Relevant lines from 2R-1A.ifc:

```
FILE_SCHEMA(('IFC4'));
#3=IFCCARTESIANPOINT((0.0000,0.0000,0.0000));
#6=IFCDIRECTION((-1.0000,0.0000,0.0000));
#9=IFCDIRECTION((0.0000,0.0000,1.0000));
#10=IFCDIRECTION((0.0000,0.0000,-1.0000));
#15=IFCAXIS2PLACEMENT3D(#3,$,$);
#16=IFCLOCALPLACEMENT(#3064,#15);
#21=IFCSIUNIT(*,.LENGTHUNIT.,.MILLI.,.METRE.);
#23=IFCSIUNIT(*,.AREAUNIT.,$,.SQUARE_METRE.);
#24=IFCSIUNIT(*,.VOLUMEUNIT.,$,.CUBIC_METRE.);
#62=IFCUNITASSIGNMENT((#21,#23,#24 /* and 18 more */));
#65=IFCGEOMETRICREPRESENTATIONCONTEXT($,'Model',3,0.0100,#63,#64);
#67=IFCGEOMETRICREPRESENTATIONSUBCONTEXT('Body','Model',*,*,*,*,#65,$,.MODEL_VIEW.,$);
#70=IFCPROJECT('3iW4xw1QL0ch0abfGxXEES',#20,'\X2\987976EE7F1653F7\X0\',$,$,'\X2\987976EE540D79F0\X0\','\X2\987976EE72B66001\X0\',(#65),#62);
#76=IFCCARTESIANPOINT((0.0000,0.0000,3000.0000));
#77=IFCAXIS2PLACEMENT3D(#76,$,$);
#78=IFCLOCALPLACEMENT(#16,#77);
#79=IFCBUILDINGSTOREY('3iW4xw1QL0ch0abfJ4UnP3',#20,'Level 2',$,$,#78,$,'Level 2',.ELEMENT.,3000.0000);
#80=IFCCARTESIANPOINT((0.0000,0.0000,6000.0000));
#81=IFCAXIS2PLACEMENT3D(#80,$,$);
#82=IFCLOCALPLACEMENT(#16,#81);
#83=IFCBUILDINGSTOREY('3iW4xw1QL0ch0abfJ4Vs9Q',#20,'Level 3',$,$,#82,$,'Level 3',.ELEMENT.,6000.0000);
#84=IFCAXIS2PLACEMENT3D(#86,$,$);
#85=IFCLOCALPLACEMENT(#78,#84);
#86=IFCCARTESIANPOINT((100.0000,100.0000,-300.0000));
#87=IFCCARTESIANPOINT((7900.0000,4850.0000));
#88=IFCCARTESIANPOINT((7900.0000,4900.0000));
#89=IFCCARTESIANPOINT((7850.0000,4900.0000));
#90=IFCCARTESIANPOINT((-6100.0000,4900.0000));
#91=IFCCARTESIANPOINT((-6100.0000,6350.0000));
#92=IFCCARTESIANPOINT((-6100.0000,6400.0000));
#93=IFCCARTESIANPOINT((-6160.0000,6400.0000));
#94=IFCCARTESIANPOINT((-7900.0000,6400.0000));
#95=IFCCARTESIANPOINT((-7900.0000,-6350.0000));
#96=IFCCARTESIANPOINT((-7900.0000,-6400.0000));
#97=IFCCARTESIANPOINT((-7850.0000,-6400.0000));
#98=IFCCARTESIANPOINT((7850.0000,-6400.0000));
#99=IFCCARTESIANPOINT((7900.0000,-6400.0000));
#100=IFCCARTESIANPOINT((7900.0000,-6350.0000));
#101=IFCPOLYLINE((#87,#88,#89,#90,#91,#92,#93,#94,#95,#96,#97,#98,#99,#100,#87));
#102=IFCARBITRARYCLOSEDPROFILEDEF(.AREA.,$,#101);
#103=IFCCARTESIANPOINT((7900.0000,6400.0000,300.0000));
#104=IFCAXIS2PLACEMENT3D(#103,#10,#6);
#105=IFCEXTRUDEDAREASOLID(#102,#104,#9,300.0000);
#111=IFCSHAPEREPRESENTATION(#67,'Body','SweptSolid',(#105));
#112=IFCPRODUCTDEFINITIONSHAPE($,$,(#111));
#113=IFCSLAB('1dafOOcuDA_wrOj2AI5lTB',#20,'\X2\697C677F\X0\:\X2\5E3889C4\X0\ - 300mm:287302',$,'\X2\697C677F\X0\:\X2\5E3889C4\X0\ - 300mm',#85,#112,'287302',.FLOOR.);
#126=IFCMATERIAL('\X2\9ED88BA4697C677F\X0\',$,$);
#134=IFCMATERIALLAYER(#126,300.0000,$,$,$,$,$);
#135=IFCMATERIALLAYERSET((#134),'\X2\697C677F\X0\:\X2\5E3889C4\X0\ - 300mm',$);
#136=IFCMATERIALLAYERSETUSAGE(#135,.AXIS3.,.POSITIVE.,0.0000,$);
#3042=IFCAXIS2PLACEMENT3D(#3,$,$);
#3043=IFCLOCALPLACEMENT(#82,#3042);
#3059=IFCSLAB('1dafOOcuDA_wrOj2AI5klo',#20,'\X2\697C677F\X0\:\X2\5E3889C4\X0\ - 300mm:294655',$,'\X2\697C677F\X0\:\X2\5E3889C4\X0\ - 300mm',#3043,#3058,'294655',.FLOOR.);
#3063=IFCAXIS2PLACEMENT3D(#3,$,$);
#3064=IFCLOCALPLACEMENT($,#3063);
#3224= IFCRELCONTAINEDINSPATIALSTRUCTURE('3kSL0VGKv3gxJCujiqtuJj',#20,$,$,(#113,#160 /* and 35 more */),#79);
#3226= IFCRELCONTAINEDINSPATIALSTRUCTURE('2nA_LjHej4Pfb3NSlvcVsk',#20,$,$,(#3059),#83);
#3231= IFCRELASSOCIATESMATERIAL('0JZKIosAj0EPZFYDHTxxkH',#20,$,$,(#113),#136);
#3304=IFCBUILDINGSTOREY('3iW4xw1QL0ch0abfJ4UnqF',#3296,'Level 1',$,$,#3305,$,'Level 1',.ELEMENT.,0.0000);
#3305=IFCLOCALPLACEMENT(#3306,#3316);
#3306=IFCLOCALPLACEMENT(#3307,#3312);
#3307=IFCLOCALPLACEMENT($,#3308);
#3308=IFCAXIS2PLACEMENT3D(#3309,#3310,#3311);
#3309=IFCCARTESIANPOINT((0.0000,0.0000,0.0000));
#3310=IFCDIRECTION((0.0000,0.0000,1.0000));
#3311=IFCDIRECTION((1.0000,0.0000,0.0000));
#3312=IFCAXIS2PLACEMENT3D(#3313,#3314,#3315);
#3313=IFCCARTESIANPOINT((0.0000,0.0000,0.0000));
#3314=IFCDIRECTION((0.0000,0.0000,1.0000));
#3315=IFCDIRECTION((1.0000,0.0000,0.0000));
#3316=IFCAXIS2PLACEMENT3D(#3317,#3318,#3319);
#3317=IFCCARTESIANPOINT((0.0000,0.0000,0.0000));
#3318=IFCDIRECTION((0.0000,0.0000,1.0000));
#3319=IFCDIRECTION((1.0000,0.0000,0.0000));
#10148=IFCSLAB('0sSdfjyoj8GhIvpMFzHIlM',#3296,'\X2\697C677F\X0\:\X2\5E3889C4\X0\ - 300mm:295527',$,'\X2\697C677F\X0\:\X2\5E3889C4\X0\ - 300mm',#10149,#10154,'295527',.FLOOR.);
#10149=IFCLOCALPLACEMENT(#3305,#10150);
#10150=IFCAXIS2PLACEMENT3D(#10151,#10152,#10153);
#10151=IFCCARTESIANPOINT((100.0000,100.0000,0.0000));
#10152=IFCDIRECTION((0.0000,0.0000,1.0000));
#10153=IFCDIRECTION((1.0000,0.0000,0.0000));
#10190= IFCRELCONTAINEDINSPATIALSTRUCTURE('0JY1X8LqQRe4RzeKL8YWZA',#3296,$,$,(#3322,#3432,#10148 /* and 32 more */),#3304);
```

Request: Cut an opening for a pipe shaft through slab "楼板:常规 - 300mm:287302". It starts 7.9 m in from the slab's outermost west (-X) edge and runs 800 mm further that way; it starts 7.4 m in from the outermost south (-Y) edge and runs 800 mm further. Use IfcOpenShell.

```python
import numpy as np
import ifcopenshell
import ifcopenshell.api.feature
import ifcopenshell.api.geometry
import ifcopenshell.api.root
import ifcopenshell.geom
import ifcopenshell.util.placement
import ifcopenshell.util.representation
import ifcopenshell.util.shape
import ifcopenshell.util.unit

model = ifcopenshell.open("2R-1A.ifc")
unit_scale = ifcopenshell.util.unit.calculate_unit_scale(model)
settings = ifcopenshell.geom.settings()


def volume(element):
    """Net volume in cubic metres, openings subtracted."""
    shape = ifcopenshell.geom.create_shape(settings, element)
    return ifcopenshell.util.shape.get_volume(shape.geometry)


slab = model.by_guid("1dafOOcuDA_wrOj2AI5lTB")
before = volume(slab)

# Extent in the slab's own axes, in metres. The edges named are its -X and -Y sides.
slab_shape = ifcopenshell.geom.create_shape(settings, slab)
vertices = ifcopenshell.util.shape.get_vertices(slab_shape.geometry)
x_min, y_min, bottom = vertices.min(axis=0)
top = vertices[:, 2].max()

opening = ifcopenshell.api.root.create_entity(model, ifc_class="IfcOpeningElement", name="Pipe shaft opening", predefined_type="OPENING")
context = ifcopenshell.util.representation.get_context(model, "Model", "Body", "MODEL_VIEW")
width, depth = 0.8, 0.8
outline = [(0.0, 0.0), (width, 0.0), (width, depth), (0.0, depth), (0.0, 0.0)]
# Overshoot both faces by 50 mm so the cut is clean.
shape = ifcopenshell.api.geometry.add_slab_representation(
    model, context=context, depth=top - bottom + 0.1, polyline=outline
)
ifcopenshell.api.geometry.assign_representation(model, product=opening, representation=shape)

matrix = ifcopenshell.util.placement.get_local_placement(slab.ObjectPlacement)
matrix[:, 3] = matrix @ np.append(np.array([x_min + 7.9, y_min + 7.4, bottom - 0.05]) / unit_scale, 1.0)
ifcopenshell.api.geometry.edit_object_placement(model, product=opening, matrix=matrix, is_si=False)
ifcopenshell.api.feature.add_feature(model, feature=opening, element=slab)

after = volume(slab)

print(f"slab volume {before:.3f} -> {after:.3f} m3")

model.write("2R-1A-out.ifc")
```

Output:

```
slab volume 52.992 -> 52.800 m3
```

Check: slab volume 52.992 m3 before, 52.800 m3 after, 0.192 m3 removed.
